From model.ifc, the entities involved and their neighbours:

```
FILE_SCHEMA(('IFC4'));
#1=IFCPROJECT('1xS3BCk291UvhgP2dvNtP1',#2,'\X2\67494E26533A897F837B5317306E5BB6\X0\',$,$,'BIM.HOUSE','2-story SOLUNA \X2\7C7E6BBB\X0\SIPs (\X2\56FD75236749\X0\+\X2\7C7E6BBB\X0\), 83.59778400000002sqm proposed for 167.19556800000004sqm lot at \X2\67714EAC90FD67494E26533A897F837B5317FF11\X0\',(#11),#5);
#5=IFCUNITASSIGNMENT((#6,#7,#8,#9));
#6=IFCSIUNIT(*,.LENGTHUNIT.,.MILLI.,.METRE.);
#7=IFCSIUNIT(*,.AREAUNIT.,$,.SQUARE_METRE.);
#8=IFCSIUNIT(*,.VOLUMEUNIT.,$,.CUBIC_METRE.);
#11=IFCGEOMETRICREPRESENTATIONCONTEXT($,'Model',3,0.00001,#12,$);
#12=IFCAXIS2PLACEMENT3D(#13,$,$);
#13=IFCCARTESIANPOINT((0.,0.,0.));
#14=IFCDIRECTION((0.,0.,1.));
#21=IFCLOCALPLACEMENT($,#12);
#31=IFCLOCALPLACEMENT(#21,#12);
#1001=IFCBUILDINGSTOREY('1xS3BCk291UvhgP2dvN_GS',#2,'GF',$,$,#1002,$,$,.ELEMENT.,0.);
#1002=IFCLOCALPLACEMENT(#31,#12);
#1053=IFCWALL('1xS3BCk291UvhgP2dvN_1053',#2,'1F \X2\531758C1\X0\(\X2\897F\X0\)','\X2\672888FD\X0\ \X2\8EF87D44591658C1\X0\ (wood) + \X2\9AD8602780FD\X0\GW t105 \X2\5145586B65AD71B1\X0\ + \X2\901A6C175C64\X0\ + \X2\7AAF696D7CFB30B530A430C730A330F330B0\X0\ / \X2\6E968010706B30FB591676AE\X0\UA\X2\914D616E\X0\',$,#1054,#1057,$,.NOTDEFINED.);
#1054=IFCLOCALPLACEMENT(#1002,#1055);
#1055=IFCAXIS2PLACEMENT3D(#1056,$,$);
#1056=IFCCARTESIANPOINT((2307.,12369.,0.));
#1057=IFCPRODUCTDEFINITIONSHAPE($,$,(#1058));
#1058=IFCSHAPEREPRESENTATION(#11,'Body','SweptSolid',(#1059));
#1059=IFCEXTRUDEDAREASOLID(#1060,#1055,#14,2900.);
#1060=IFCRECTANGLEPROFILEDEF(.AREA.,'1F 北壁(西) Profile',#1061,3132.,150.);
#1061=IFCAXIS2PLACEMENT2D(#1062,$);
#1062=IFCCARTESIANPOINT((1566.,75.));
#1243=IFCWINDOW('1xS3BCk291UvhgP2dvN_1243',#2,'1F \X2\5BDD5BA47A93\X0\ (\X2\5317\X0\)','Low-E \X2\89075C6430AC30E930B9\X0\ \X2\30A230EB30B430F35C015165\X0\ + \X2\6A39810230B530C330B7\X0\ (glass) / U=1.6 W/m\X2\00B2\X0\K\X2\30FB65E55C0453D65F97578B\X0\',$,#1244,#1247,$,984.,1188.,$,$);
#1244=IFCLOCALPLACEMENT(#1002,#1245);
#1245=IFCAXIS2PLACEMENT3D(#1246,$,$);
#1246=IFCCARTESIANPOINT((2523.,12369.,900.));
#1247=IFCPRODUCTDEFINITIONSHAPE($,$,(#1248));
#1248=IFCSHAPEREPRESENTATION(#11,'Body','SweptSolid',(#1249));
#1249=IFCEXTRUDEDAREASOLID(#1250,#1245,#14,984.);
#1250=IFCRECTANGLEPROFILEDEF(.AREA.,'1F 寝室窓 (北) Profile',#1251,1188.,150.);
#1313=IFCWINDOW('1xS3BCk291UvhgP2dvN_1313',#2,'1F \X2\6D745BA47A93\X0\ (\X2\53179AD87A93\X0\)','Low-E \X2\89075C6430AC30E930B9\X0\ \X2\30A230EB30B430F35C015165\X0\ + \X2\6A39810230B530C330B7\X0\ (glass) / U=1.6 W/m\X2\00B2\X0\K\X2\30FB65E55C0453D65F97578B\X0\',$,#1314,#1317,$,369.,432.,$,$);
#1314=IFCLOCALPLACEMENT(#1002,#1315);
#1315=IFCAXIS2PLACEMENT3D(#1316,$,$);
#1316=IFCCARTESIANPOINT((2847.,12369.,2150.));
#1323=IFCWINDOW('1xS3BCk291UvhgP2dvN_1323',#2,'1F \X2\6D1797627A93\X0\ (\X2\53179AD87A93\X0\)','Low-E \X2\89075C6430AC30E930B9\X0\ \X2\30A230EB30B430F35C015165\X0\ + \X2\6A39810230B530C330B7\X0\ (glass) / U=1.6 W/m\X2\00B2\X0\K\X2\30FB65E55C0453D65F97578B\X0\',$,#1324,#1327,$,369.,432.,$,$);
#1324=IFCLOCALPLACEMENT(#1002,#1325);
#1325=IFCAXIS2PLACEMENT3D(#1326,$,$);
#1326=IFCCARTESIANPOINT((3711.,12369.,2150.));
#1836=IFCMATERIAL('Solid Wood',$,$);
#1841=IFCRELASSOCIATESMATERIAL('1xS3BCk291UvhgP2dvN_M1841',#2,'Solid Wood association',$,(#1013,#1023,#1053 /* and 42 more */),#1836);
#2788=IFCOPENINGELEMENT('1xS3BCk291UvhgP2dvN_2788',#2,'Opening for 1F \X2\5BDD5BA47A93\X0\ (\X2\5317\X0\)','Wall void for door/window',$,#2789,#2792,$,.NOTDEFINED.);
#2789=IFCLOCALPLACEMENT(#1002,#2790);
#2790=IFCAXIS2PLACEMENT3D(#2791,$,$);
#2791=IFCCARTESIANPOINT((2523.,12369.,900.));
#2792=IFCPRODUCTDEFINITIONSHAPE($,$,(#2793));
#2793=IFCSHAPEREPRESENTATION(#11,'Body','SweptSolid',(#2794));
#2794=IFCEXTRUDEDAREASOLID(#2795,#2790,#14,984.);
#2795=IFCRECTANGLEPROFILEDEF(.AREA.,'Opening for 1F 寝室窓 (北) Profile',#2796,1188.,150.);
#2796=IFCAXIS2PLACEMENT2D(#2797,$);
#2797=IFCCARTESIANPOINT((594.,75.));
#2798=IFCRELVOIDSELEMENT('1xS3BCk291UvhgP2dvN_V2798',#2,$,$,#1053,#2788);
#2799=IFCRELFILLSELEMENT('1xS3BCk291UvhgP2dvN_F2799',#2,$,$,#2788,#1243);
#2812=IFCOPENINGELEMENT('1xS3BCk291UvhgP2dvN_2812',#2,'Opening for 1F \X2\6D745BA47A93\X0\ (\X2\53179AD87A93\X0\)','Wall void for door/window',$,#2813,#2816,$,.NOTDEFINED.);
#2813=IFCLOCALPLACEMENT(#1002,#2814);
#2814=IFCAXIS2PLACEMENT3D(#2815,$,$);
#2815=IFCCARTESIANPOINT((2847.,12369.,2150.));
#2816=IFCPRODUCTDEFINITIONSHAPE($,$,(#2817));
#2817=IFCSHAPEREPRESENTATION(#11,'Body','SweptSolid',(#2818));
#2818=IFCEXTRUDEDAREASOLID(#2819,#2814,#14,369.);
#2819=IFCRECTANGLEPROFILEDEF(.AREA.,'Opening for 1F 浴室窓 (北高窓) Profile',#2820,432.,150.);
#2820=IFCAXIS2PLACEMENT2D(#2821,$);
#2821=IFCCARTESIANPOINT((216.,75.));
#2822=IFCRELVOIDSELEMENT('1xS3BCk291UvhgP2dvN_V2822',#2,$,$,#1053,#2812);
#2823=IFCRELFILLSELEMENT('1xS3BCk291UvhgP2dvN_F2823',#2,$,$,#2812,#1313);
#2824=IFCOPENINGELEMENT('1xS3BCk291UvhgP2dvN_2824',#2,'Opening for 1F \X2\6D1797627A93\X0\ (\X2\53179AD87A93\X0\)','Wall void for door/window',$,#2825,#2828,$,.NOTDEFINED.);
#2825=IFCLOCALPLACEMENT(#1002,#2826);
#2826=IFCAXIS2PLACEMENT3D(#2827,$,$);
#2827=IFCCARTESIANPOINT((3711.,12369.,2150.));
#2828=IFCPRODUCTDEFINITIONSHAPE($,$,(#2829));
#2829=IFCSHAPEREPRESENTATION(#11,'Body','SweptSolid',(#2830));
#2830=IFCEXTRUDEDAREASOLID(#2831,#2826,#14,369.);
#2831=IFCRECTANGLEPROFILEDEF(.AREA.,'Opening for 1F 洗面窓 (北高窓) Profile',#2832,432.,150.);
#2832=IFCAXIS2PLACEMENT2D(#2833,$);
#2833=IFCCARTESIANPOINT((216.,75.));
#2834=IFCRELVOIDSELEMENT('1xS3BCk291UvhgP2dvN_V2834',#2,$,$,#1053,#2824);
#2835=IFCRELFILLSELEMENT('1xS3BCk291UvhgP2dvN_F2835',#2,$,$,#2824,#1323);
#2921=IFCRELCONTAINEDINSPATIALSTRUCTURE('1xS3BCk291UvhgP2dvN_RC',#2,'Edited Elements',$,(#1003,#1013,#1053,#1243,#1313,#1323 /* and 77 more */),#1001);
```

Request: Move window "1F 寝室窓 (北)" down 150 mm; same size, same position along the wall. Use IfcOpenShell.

```python
import numpy as np
import ifcopenshell
import ifcopenshell.api.geometry
import ifcopenshell.util.placement
import ifcopenshell.util.unit

model = ifcopenshell.open("model.ifc")
unit_scale = ifcopenshell.util.unit.calculate_unit_scale(model)

window = model.by_guid("1xS3BCk291UvhgP2dvN_1243")
opening = window.FillsVoids[0].RelatingOpeningElement
dz = -0.15 / unit_scale

shift = np.array([0.0, 0.0, dz])
# The window is not placed relative to its opening, so move both.
for product in (opening, window):
    matrix = ifcopenshell.util.placement.get_local_placement(product.ObjectPlacement)
    matrix[:3, 3] += shift
    ifcopenshell.api.geometry.edit_object_placement(model, product=product, matrix=matrix, is_si=False)

print(f"moved by {dz * unit_scale:+.3f} m")

model.write("model-out.ifc")
```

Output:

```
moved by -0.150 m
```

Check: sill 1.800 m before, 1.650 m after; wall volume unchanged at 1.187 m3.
